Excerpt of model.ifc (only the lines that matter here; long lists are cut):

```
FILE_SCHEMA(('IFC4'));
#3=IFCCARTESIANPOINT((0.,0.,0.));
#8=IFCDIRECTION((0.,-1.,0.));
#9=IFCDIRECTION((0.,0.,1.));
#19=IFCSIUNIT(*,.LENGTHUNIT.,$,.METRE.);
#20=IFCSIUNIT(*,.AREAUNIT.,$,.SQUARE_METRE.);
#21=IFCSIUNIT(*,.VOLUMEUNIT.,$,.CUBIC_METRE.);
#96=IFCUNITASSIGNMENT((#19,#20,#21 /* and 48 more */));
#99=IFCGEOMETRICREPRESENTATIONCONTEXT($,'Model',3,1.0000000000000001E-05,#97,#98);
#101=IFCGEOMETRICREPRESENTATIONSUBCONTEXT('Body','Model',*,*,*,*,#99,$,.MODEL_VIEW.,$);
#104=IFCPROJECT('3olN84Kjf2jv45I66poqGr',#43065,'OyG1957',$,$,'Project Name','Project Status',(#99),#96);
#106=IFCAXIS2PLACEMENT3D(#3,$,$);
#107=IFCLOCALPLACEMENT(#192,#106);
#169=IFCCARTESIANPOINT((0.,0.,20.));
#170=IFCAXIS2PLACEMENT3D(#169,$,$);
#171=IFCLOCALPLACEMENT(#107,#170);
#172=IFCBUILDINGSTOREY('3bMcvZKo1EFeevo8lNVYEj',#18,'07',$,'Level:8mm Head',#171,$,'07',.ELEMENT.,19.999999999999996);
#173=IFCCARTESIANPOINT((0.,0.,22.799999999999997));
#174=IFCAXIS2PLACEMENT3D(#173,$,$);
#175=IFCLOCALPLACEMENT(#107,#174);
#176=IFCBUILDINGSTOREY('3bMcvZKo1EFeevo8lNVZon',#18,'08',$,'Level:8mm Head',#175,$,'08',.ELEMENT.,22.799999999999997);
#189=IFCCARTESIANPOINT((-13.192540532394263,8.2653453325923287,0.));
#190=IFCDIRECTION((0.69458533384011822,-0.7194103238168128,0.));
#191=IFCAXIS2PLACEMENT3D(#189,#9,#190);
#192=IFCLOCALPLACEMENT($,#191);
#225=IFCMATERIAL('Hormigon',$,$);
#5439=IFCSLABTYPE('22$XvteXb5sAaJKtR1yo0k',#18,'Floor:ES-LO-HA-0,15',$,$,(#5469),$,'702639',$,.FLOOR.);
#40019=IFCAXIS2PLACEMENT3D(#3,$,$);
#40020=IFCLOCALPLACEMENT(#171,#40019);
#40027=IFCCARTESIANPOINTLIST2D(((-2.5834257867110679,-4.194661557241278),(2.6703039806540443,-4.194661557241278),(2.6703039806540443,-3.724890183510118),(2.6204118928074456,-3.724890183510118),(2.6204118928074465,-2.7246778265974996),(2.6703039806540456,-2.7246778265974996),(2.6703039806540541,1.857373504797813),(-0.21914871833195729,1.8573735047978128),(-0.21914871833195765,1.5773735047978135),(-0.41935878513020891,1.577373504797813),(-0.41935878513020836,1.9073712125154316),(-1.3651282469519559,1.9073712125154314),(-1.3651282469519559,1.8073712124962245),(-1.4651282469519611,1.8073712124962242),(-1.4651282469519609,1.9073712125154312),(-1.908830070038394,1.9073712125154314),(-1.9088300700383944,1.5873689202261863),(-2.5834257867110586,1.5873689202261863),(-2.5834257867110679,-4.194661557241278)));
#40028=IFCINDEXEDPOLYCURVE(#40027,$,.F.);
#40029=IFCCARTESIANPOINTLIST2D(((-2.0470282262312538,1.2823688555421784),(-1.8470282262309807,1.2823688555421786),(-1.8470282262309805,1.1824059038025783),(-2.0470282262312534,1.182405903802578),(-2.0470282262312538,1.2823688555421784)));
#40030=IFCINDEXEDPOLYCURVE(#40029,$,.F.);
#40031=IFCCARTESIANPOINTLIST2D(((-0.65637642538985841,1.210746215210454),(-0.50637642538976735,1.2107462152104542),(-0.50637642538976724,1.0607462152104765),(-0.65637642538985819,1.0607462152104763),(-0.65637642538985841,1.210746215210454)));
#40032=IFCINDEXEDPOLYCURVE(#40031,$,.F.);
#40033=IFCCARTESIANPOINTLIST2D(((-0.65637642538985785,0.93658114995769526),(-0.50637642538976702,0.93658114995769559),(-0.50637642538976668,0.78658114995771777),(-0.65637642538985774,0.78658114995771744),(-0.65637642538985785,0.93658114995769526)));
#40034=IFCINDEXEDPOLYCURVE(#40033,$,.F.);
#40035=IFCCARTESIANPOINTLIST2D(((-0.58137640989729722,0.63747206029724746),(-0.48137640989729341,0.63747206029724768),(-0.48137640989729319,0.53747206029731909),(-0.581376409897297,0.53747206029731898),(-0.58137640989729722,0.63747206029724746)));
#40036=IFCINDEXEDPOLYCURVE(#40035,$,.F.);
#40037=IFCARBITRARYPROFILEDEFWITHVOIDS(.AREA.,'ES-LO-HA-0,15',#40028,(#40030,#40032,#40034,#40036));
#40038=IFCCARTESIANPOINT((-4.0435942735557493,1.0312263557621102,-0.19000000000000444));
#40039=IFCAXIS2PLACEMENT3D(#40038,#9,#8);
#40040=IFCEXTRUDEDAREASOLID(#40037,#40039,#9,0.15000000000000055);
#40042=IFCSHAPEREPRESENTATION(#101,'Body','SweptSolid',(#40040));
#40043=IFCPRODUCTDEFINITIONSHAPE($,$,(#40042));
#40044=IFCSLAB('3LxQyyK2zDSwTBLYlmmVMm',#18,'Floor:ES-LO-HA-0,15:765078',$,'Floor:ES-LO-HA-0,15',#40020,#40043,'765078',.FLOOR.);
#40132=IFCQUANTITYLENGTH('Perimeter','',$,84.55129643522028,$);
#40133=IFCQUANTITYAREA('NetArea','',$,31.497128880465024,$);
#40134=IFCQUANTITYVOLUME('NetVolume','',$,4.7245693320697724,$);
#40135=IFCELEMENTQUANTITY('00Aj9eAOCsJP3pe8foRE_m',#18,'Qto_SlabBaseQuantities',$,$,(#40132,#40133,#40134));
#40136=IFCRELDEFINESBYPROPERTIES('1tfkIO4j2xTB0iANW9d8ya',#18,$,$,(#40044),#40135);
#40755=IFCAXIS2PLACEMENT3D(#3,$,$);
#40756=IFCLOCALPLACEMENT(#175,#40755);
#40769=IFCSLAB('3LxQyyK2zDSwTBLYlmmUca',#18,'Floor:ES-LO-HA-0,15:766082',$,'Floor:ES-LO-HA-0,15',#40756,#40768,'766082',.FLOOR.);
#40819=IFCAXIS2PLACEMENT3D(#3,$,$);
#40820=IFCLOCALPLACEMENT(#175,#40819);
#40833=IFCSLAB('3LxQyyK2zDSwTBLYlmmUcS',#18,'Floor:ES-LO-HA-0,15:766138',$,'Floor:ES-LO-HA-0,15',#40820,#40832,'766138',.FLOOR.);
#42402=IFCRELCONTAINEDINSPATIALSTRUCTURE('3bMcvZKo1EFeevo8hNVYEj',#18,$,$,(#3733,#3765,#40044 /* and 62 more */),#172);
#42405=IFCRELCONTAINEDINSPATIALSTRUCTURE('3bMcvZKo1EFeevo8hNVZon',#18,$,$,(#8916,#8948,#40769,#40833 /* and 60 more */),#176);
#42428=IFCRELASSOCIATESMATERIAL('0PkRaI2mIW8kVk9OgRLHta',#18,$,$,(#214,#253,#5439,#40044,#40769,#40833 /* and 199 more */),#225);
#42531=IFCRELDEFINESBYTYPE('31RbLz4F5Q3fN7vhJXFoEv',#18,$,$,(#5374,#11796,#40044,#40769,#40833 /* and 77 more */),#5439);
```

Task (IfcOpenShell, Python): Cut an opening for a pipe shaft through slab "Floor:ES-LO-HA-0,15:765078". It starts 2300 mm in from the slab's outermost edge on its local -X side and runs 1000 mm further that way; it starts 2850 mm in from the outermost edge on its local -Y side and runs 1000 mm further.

```python
import numpy as np
import ifcopenshell
import ifcopenshell.api.feature
import ifcopenshell.api.geometry
import ifcopenshell.api.pset
import ifcopenshell.api.root
import ifcopenshell.geom
import ifcopenshell.util.element
import ifcopenshell.util.placement
import ifcopenshell.util.representation
import ifcopenshell.util.shape
import ifcopenshell.util.unit

model = ifcopenshell.open("model.ifc")
unit_scale = ifcopenshell.util.unit.calculate_unit_scale(model)
area_scale = ifcopenshell.util.unit.calculate_unit_scale(model, "AREAUNIT")
volume_scale = ifcopenshell.util.unit.calculate_unit_scale(model, "VOLUMEUNIT")
settings = ifcopenshell.geom.settings()


def volume(element):
    """Net volume in cubic metres, openings subtracted."""
    shape = ifcopenshell.geom.create_shape(settings, element)
    return ifcopenshell.util.shape.get_volume(shape.geometry)


slab = model.by_id(40044)
before = volume(slab)

# Extent in the slab's own axes, in metres. The edges named are its -X and -Y sides.
slab_shape = ifcopenshell.geom.create_shape(settings, slab)
vertices = ifcopenshell.util.shape.get_vertices(slab_shape.geometry)
x_min, y_min, bottom = vertices.min(axis=0)
top = vertices[:, 2].max()

opening = ifcopenshell.api.root.create_entity(model, ifc_class="IfcOpeningElement", name="Pipe shaft opening", predefined_type="OPENING")
context = ifcopenshell.util.representation.get_context(model, "Model", "Body", "MODEL_VIEW")
width, depth = 1, 1
outline = [(0.0, 0.0), (width, 0.0), (width, depth), (0.0, depth), (0.0, 0.0)]
# Overshoot both faces by 50 mm so the cut is clean.
shape = ifcopenshell.api.geometry.add_slab_representation(
    model, context=context, depth=top - bottom + 0.1, polyline=outline
)
ifcopenshell.api.geometry.assign_representation(model, product=opening, representation=shape)

matrix = ifcopenshell.util.placement.get_local_placement(slab.ObjectPlacement)
matrix[:, 3] = matrix @ np.append(np.array([x_min + 2.3, y_min + 2.85, bottom - 0.05]) / unit_scale, 1.0)
ifcopenshell.api.geometry.edit_object_placement(model, product=opening, matrix=matrix, is_si=False)
ifcopenshell.api.feature.add_feature(model, feature=opening, element=slab)

after = volume(slab)

# Update the slab's stored quantities.
qto = model.by_id(ifcopenshell.util.element.get_pset(slab, "Qto_SlabBaseQuantities", should_inherit=False)["id"])
ifcopenshell.api.pset.edit_qto(model, qto=qto, properties={
    "NetArea": after / (top - bottom) / area_scale,
    "NetVolume": after / volume_scale,
})

print(f"slab volume {before:.3f} -> {after:.3f} m3")

model.write("model_v2.ifc")
```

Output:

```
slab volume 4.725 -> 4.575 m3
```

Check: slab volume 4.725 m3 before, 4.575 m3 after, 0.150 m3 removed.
